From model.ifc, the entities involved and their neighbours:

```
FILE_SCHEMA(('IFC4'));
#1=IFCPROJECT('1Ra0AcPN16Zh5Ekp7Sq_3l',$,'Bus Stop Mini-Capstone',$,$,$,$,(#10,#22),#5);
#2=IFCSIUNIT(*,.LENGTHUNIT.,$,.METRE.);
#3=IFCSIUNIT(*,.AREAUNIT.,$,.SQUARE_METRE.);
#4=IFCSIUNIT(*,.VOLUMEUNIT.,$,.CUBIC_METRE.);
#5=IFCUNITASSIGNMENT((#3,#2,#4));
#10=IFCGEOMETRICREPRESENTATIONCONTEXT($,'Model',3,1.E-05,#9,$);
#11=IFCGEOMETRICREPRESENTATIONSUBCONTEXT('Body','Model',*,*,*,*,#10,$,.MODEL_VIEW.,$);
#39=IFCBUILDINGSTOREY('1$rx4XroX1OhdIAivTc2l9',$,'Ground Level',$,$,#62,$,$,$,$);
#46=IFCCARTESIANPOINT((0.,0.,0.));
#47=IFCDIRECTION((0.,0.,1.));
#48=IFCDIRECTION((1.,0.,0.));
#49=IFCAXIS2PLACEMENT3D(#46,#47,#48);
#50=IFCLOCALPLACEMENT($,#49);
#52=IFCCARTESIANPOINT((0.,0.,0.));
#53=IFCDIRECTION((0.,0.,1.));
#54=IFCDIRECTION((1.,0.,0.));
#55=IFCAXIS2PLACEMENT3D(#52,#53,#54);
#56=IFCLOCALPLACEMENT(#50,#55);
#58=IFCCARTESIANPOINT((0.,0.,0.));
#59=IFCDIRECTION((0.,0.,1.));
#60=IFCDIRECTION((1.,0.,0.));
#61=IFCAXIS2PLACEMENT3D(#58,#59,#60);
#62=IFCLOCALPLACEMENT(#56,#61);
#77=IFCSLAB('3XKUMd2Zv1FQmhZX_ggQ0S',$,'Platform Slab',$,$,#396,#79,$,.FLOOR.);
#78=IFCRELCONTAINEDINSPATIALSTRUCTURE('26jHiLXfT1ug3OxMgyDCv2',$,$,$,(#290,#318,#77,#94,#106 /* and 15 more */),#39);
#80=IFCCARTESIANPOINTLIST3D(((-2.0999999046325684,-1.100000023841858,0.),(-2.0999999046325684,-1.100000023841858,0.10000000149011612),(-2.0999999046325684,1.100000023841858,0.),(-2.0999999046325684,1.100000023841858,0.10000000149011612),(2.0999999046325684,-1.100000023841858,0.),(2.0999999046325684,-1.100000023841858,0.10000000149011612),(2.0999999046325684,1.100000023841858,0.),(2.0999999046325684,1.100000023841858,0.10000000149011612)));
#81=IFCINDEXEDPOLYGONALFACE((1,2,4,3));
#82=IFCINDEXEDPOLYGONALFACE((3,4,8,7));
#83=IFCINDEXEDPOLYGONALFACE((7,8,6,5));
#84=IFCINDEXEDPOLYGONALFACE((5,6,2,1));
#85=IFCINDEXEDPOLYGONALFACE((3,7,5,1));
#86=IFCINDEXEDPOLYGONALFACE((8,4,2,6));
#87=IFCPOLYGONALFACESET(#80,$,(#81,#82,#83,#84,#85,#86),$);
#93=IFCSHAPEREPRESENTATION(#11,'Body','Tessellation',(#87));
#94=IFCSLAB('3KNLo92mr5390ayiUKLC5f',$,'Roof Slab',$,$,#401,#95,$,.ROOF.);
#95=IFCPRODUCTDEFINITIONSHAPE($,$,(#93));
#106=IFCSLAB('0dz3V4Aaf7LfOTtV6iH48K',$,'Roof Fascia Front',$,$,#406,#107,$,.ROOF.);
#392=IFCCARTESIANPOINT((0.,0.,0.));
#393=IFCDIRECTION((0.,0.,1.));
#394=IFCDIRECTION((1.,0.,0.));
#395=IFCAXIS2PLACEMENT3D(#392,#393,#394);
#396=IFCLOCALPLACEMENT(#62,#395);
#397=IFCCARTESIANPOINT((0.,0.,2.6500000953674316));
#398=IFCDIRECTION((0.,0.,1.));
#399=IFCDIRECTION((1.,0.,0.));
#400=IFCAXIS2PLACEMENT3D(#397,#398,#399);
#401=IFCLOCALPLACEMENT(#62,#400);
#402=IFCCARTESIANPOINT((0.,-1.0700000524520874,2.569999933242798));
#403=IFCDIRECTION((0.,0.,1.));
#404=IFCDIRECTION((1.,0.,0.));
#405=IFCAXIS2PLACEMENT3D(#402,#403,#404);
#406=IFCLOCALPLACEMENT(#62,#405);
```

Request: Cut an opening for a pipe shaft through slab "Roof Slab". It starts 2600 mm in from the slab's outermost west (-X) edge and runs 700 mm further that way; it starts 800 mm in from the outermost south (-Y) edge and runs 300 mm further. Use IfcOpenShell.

```python
import numpy as np
import ifcopenshell
import ifcopenshell.api.feature
import ifcopenshell.api.geometry
import ifcopenshell.api.root
import ifcopenshell.geom
import ifcopenshell.util.placement
import ifcopenshell.util.representation
import ifcopenshell.util.shape
import ifcopenshell.util.unit

model = ifcopenshell.open("model.ifc")
unit_scale = ifcopenshell.util.unit.calculate_unit_scale(model)
settings = ifcopenshell.geom.settings()


def volume(element):
    """Net volume in cubic metres, openings subtracted."""
    shape = ifcopenshell.geom.create_shape(settings, element)
    return ifcopenshell.util.shape.get_volume(shape.geometry)


slab = model.by_guid("3KNLo92mr5390ayiUKLC5f")
before = volume(slab)

# Extent in the slab's own axes, in metres. The edges named are its -X and -Y sides.
slab_shape = ifcopenshell.geom.create_shape(settings, slab)
vertices = ifcopenshell.util.shape.get_vertices(slab_shape.geometry)
x_min, y_min, bottom = vertices.min(axis=0)
top = vertices[:, 2].max()

opening = ifcopenshell.api.root.create_entity(model, ifc_class="IfcOpeningElement", name="Pipe shaft opening", predefined_type="OPENING")
context = ifcopenshell.util.representation.get_context(model, "Model", "Body", "MODEL_VIEW")
width, depth = 0.7, 0.3
outline = [(0.0, 0.0), (width, 0.0), (width, depth), (0.0, depth), (0.0, 0.0)]
# Overshoot both faces by 50 mm so the cut is clean.
shape = ifcopenshell.api.geometry.add_slab_representation(
    model, context=context, depth=top - bottom + 0.1, polyline=outline
)
ifcopenshell.api.geometry.assign_representation(model, product=opening, representation=shape)

matrix = ifcopenshell.util.placement.get_local_placement(slab.ObjectPlacement)
matrix[:, 3] = matrix @ np.append(np.array([x_min + 2.6, y_min + 0.8, bottom - 0.05]) / unit_scale, 1.0)
ifcopenshell.api.geometry.edit_object_placement(model, product=opening, matrix=matrix, is_si=False)
ifcopenshell.api.feature.add_feature(model, feature=opening, element=slab)

after = volume(slab)

print(f"slab volume {before:.3f} -> {after:.3f} m3")

model.write("model_updated.ifc")
```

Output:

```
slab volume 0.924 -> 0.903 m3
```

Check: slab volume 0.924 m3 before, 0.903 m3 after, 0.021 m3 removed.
